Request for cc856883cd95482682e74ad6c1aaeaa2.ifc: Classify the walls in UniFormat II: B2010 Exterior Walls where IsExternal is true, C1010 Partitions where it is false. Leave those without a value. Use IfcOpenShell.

First a look at what the model holds.

```python
import ifcopenshell
import ifcopenshell.util.element

model = ifcopenshell.open("cc856883cd95482682e74ad6c1aaeaa2.ifc")
print(model.schema)
print("classifications:", [c.Name for c in model.by_type("IfcClassification")])
values = [ifcopenshell.util.element.get_pset(e, "Pset_WallCommon", "IsExternal") for e in model.by_type("IfcWall")]
for value in (True, False, None):
    print("IsExternal", value, values.count(value))
```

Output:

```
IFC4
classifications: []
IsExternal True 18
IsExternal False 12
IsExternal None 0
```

```python
import ifcopenshell
import ifcopenshell.api.classification
import ifcopenshell.util.element

model = ifcopenshell.open("cc856883cd95482682e74ad6c1aaeaa2.ifc")

system = ifcopenshell.api.classification.add_classification(model, classification="UniFormat II")

walls = model.by_type("IfcWall")
external = {e: ifcopenshell.util.element.get_pset(e, "Pset_WallCommon", "IsExternal") for e in walls}
for flag, code, name in ((True, "B2010", "Exterior Walls"), (False, "C1010", "Partitions")):
    products = [e for e in walls if external[e] is flag]
    ifcopenshell.api.classification.add_reference(
        model, products=products, classification=system, identification=code, name=name
    )
    print(code, len(products))

model.write("cc856883cd95482682e74ad6c1aaeaa2_edited.ifc")
```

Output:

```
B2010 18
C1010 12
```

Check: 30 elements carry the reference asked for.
